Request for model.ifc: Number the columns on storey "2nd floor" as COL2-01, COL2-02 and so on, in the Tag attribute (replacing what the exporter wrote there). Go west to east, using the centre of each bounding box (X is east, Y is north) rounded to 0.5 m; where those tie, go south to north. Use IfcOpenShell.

First a look at what the model holds.

```python
import ifcopenshell
import ifcopenshell.util.element
import ifcopenshell.util.placement

model = ifcopenshell.open("model.ifc")
print(model.schema)
storey = next(s for s in model.by_type("IfcBuildingStorey") if s.Name == "2nd floor")
columns = [e for e in ifcopenshell.util.element.get_decomposition(storey) if e.is_a("IfcColumn")]
for e in sorted(columns, key=lambda e: e.id()):
    origin = ifcopenshell.util.placement.get_local_placement(e.ObjectPlacement)[:3, 3]
    print(e.id(), e.Tag, e.Name, origin.round(2) + 0.0, sep=" | ")
```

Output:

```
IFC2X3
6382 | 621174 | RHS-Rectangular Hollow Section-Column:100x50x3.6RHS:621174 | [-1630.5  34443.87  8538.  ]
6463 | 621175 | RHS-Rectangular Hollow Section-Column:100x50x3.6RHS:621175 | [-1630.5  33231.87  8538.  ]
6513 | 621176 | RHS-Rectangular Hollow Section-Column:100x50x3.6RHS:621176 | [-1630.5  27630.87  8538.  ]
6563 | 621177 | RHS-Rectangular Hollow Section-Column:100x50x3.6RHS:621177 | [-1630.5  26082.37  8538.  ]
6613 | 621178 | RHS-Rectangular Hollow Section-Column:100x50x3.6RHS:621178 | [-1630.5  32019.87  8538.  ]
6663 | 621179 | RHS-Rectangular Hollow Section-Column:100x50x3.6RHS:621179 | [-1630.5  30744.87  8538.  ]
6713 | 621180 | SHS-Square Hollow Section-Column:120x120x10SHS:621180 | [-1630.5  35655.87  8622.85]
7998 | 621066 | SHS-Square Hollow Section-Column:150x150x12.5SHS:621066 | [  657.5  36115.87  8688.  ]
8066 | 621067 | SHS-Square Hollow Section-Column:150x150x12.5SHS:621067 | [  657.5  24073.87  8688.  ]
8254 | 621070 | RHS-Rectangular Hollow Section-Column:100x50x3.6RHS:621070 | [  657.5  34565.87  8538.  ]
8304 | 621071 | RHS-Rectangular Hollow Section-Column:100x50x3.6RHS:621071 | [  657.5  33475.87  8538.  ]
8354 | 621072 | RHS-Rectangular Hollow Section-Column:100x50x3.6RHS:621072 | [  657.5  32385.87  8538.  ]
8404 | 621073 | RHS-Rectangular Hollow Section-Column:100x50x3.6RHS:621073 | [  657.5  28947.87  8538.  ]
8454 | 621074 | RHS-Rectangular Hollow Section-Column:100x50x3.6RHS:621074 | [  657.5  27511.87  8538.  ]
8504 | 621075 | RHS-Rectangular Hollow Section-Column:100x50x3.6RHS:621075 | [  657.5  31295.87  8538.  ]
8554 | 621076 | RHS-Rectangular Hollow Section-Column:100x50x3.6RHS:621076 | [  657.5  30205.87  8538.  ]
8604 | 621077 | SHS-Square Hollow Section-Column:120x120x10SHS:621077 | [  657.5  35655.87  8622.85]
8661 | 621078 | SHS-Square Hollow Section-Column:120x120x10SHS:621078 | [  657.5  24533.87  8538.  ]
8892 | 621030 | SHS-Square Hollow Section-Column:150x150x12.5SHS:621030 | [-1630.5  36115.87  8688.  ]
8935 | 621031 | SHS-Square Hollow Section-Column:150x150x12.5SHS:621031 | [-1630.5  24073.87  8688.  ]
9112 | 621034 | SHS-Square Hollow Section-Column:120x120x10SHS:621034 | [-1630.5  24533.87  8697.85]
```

```python
import ifcopenshell
import ifcopenshell.geom
import ifcopenshell.util.element
import ifcopenshell.util.shape

model = ifcopenshell.open("model.ifc")
settings = ifcopenshell.geom.settings()
settings.set("use-world-coords", True)


def centre(element):
    shape = ifcopenshell.geom.create_shape(settings, element)
    return ifcopenshell.util.shape.get_bbox_centroid(shape.geometry)


storey = next(s for s in model.by_type("IfcBuildingStorey") if s.Name == "2nd floor")
columns = [e for e in ifcopenshell.util.element.get_decomposition(storey) if e.is_a("IfcColumn")]

# Insertion points can sit at a corner or the storey origin, so sort by the geometry (in metres).
centres = {e: centre(e) for e in columns}
columns.sort(key=lambda e: (round(centres[e][0] / 0.5), centres[e][1]))

for i, e in enumerate(columns, start=1):
    number = f"COL2-{i:02d}"
    e.Tag = number
    print(e.id(), number)

model.write("model_edited.ifc")
```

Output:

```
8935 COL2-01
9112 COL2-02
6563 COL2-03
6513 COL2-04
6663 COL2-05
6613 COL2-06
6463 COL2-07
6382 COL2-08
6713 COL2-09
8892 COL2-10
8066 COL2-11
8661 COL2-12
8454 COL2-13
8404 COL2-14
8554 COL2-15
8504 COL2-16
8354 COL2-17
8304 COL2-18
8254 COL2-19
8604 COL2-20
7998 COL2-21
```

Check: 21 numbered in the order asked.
